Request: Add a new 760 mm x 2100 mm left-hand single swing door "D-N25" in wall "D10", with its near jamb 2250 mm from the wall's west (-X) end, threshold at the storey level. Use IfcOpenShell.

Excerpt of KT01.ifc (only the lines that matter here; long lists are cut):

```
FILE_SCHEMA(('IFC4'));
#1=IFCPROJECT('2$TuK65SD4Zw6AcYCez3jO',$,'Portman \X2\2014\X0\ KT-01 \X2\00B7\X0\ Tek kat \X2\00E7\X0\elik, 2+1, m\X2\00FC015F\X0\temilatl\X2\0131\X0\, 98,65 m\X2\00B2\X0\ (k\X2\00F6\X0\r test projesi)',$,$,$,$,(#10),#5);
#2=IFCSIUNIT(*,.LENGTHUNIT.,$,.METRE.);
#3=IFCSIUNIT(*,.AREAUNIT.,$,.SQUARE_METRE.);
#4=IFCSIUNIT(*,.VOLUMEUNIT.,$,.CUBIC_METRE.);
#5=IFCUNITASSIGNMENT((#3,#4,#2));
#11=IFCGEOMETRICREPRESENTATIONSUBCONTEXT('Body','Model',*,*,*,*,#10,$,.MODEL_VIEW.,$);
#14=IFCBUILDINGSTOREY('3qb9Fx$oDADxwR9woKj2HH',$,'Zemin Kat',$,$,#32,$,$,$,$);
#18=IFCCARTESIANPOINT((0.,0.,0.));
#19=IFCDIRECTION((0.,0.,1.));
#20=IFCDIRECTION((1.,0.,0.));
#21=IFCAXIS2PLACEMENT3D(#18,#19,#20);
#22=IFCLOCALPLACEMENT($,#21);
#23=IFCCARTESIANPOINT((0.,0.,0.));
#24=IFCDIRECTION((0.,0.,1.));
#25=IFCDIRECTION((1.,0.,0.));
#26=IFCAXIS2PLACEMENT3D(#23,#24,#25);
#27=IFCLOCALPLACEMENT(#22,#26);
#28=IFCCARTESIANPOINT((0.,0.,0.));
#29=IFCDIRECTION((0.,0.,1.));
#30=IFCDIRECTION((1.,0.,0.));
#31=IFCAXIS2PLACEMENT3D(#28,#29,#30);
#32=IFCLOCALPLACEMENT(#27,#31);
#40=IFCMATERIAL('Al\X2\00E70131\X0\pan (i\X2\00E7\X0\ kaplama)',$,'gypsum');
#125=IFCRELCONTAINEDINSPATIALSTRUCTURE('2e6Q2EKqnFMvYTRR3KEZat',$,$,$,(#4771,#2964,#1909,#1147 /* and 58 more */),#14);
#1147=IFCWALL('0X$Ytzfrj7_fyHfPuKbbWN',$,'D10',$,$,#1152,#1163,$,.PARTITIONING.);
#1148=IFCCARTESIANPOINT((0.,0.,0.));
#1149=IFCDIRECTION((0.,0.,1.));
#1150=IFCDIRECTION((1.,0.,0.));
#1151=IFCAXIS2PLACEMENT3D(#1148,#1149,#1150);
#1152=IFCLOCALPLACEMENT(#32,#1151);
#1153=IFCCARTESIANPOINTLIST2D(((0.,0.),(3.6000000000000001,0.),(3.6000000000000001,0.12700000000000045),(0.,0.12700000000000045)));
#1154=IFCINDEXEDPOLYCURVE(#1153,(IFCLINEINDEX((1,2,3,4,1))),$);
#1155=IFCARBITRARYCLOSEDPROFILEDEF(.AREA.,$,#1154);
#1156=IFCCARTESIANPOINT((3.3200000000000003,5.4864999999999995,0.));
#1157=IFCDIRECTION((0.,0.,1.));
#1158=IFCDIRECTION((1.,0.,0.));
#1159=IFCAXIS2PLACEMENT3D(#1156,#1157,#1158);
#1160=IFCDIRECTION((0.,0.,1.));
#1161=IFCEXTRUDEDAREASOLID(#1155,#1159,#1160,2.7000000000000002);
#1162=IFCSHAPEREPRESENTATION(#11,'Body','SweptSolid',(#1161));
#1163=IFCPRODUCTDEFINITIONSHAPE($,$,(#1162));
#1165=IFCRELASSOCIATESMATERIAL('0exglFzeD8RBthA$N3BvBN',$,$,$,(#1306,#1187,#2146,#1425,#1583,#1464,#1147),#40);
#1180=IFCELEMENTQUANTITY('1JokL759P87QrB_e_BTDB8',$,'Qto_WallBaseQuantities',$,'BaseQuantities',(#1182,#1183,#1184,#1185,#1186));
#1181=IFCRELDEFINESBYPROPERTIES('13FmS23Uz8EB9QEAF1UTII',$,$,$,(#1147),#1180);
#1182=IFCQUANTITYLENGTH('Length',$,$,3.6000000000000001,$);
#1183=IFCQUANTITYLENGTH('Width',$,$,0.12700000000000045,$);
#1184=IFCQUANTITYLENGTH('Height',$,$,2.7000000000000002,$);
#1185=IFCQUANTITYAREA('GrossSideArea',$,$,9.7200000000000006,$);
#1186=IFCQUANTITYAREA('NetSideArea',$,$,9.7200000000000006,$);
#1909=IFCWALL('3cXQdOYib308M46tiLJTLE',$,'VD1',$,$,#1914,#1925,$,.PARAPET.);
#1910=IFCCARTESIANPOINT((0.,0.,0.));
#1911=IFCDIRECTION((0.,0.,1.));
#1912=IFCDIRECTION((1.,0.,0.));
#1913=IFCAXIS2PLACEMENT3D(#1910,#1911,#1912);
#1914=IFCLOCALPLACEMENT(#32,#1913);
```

```python
import numpy as np
import ifcopenshell
import ifcopenshell.api.feature
import ifcopenshell.api.geometry
import ifcopenshell.api.pset
import ifcopenshell.api.root
import ifcopenshell.api.spatial
import ifcopenshell.geom
import ifcopenshell.util.element
import ifcopenshell.util.placement
import ifcopenshell.util.representation
import ifcopenshell.util.shape
import ifcopenshell.util.unit

model = ifcopenshell.open("KT01.ifc")
unit_scale = ifcopenshell.util.unit.calculate_unit_scale(model)
area_scale = ifcopenshell.util.unit.calculate_unit_scale(model, "AREAUNIT")
settings = ifcopenshell.geom.settings()


def volume(element):
    """Net volume in cubic metres, openings subtracted."""
    shape = ifcopenshell.geom.create_shape(settings, element)
    return ifcopenshell.util.shape.get_volume(shape.geometry)


wall = model.by_id(1147)
storey = ifcopenshell.util.element.get_container(wall, ifc_class="IfcBuildingStorey")
context = ifcopenshell.util.representation.get_context(model, "Model", "Body", "MODEL_VIEW")
before = volume(wall)

width, height, from_end, sill = 0.76, 2.1, 2.25, 0.0  # metres

# The wall runs along its own X axis, and the end named is its -X end.
wall_shape = ifcopenshell.geom.create_shape(settings, wall)
x, y, z = ifcopenshell.util.shape.get_vertices(wall_shape.geometry).T
start = x.min() + from_end
face, thickness = float(y.min()), float(y.max() - y.min())
wall_matrix = ifcopenshell.util.placement.get_local_placement(wall.ObjectPlacement)
level = ifcopenshell.util.placement.get_local_placement(storey.ObjectPlacement)[2, 3]


def in_wall(x, y):
    """Placement at x, y metres in the wall's axes, at sill height."""
    matrix = wall_matrix.copy()
    matrix[:, 3] = wall_matrix @ np.array([x / unit_scale, y / unit_scale, 0.0, 1.0])
    matrix[2, 3] = level + sill / unit_scale
    return matrix


# Opening: a box that overshoots both wall faces by 50 mm.
opening = ifcopenshell.api.root.create_entity(model, ifc_class="IfcOpeningElement", predefined_type="OPENING")
box = ifcopenshell.api.geometry.add_wall_representation(
    model, context=context, length=width, height=height, thickness=thickness + 0.1
)
ifcopenshell.api.geometry.assign_representation(model, product=opening, representation=box)
ifcopenshell.api.geometry.edit_object_placement(model, product=opening, matrix=in_wall(start, face - 0.05), is_si=False)
ifcopenshell.api.feature.add_feature(model, feature=opening, element=wall)

door = ifcopenshell.api.root.create_entity(model, ifc_class="IfcDoor", name="D-N25", predefined_type="DOOR")
door.OverallWidth, door.OverallHeight = width / unit_scale, height / unit_scale
door.OperationType = "SINGLE_SWING_LEFT"
body = ifcopenshell.api.geometry.add_door_representation(
    model,
    context=context,
    overall_width=door.OverallWidth,
    overall_height=door.OverallHeight,
    operation_type="SINGLE_SWING_LEFT",
    lining_properties={"LiningDepth": thickness / unit_scale, "ThresholdDepth": thickness / unit_scale},
)
ifcopenshell.api.geometry.assign_representation(model, product=door, representation=body)
ifcopenshell.api.spatial.assign_container(model, products=[door], relating_structure=storey)
ifcopenshell.api.feature.add_filling(model, opening=opening, element=door)

# The lining spans the wall, so the door starts at the wall face.
ifcopenshell.api.geometry.edit_object_placement(model, product=door, matrix=in_wall(start, face), is_si=False)

after = volume(wall)

# Update the wall's stored quantities.
qto = model.by_id(ifcopenshell.util.element.get_pset(wall, "Qto_WallBaseQuantities", should_inherit=False)["id"])
ifcopenshell.api.pset.edit_qto(model, qto=qto, properties={"NetSideArea": after / thickness / area_scale})

print(f"wall volume {before:.3f} -> {after:.3f} m3")

model.write("KT01_v2.ifc")
```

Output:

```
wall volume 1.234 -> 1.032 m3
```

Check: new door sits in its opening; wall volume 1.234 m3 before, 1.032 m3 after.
